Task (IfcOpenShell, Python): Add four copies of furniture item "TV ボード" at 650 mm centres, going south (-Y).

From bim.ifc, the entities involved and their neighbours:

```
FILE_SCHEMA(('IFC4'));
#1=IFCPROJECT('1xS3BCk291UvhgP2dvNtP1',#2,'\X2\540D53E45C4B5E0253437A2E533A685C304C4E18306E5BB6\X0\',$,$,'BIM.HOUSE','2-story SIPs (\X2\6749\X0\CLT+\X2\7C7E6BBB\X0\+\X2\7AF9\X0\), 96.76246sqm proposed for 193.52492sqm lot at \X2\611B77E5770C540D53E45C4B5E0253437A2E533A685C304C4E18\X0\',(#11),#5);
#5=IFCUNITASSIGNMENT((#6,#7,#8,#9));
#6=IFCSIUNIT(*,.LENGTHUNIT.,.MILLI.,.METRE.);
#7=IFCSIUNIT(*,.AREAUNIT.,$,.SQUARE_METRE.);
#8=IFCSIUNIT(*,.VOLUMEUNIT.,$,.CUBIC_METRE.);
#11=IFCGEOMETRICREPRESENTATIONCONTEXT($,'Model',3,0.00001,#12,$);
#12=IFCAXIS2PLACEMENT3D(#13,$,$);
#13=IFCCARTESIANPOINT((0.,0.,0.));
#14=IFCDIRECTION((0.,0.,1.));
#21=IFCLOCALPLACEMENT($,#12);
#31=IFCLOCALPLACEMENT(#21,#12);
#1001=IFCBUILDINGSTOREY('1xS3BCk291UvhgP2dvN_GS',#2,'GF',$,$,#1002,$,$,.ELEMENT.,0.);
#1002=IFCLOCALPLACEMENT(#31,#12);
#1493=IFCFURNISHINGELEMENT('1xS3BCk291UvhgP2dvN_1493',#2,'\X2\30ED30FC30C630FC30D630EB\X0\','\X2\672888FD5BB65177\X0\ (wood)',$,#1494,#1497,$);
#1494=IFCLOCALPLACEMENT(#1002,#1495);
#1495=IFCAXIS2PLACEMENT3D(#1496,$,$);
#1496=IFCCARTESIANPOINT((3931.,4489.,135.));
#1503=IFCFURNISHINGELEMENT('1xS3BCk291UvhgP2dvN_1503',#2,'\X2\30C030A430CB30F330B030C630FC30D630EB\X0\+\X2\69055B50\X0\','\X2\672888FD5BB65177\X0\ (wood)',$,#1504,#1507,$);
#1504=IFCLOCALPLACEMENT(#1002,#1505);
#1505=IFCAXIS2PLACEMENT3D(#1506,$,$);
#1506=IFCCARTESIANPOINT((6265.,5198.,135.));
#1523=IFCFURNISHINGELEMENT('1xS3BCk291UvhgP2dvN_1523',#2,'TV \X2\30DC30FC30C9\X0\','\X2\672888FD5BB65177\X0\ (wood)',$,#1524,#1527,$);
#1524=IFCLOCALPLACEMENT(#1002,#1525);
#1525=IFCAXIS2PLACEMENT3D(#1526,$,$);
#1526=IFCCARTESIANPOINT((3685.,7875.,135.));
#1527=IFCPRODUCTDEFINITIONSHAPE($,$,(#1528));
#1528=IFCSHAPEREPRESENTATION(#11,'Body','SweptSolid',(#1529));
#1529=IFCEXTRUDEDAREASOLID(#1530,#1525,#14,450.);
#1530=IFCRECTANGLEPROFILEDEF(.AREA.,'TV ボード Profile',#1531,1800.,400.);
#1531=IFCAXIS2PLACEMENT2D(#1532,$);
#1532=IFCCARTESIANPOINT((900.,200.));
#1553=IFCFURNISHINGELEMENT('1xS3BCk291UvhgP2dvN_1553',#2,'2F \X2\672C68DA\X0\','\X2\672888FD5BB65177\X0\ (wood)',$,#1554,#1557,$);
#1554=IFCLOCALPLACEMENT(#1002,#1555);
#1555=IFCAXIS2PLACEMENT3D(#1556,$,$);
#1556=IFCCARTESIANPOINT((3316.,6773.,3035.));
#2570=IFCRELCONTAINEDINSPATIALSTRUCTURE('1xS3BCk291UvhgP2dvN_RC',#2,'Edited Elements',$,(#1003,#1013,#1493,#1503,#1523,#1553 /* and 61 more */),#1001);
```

```python
import numpy as np
import ifcopenshell
import ifcopenshell.api.geometry
import ifcopenshell.api.root
import ifcopenshell.util.element
import ifcopenshell.util.placement

model = ifcopenshell.open("bim.ifc")


def reuse_history(source, copy):
    """copy_class also copies each property set's owner history, people and application; keep the originals."""
    for rel in copy.IsDefinedBy:
        if rel.is_a("IfcRelDefinesByProperties") and (history := rel.RelatingPropertyDefinition.OwnerHistory):
            rel.RelatingPropertyDefinition.OwnerHistory = source.OwnerHistory
            ifcopenshell.util.element.remove_deep2(model, history)


source = model.by_guid("1xS3BCk291UvhgP2dvN_1523")
base = ifcopenshell.util.placement.get_local_placement(source.ObjectPlacement)
step = np.array([0.0, -1.0, 0.0]) * 650.0

for i in range(1, 5):
    copy = ifcopenshell.api.root.copy_class(model, product=source)
    copy.Representation = ifcopenshell.util.element.copy_deep(
        model, source.Representation, exclude=["IfcGeometricRepresentationContext", "IfcRepresentationMap"]
    )
    reuse_history(source, copy)
    matrix = base.copy()
    matrix[:3, 3] += i * step
    print("added at", matrix[:3, 3].round(3) + 0.0)
    ifcopenshell.api.geometry.edit_object_placement(model, product=copy, matrix=matrix, is_si=False)

model.write("bim-out.ifc")
```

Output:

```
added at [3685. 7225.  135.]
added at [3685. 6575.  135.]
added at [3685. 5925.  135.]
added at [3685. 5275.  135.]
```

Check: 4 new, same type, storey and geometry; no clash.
